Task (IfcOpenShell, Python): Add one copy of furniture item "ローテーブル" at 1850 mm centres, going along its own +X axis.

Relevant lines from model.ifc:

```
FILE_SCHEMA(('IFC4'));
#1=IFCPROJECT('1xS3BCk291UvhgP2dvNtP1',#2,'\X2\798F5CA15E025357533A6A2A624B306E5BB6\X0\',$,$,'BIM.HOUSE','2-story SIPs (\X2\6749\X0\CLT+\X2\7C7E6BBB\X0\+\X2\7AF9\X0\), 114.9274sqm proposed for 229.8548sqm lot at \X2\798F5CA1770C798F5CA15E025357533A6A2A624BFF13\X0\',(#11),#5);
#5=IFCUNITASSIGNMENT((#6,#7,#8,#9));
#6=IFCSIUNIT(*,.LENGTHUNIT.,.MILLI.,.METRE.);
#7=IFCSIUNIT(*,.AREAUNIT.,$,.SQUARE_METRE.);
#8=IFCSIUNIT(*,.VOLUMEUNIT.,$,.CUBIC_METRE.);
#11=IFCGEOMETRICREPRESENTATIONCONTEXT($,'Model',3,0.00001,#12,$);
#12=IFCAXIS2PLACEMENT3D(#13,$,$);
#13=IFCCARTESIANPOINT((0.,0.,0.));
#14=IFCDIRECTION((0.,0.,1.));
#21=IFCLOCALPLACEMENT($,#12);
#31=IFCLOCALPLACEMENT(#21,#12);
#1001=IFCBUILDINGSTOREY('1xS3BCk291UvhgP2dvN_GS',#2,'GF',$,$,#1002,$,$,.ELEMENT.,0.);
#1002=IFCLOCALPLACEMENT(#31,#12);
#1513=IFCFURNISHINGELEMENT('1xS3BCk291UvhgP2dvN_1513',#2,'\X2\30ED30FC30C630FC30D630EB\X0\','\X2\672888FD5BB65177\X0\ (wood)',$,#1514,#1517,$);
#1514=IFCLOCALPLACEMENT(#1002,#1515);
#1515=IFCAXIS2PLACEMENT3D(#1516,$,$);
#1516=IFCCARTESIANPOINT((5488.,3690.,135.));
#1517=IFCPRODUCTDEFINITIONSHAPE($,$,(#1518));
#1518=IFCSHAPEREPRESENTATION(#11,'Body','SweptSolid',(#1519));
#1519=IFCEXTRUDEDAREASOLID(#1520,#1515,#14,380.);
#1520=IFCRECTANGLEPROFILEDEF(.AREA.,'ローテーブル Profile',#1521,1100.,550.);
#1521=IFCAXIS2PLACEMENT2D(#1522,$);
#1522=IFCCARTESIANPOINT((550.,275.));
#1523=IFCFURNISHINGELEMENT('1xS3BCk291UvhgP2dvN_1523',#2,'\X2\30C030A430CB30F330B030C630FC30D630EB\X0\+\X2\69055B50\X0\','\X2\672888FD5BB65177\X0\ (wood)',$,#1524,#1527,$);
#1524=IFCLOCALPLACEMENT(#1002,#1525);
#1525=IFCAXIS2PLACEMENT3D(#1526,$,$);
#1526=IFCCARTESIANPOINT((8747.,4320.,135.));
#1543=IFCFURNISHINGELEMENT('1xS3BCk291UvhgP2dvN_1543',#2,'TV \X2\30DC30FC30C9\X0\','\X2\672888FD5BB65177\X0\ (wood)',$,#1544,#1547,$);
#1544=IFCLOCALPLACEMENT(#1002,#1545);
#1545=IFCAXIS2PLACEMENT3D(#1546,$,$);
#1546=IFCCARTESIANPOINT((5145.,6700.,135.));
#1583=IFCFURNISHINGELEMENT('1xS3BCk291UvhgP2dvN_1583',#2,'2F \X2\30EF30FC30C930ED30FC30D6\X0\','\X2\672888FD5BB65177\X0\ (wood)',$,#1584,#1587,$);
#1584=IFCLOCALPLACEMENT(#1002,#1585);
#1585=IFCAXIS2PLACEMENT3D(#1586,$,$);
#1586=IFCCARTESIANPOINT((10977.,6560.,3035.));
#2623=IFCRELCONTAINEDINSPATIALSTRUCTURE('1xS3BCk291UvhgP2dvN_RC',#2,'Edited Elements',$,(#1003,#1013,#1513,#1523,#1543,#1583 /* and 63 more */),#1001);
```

```python
import ifcopenshell
import ifcopenshell.api.geometry
import ifcopenshell.api.root
import ifcopenshell.util.element
import ifcopenshell.util.placement
import ifcopenshell.util.unit

model = ifcopenshell.open("model.ifc")
unit_scale = ifcopenshell.util.unit.calculate_unit_scale(model)


def reuse_history(source, copy):
    """copy_class also copies each property set's owner history, people and application; keep the originals."""
    for rel in copy.IsDefinedBy:
        if rel.is_a("IfcRelDefinesByProperties") and (history := rel.RelatingPropertyDefinition.OwnerHistory):
            rel.RelatingPropertyDefinition.OwnerHistory = source.OwnerHistory
            ifcopenshell.util.element.remove_deep2(model, history)


source = model.by_guid("1xS3BCk291UvhgP2dvN_1513")
base = ifcopenshell.util.placement.get_local_placement(source.ObjectPlacement)
step = base[:3, 0] * 1.85 / unit_scale

for i in range(1, 2):
    copy = ifcopenshell.api.root.copy_class(model, product=source)
    copy.Representation = ifcopenshell.util.element.copy_deep(
        model, source.Representation, exclude=["IfcGeometricRepresentationContext", "IfcRepresentationMap"]
    )
    reuse_history(source, copy)
    matrix = base.copy()
    matrix[:3, 3] += i * step
    print("added at", matrix[:3, 3].round(3) + 0.0)
    ifcopenshell.api.geometry.edit_object_placement(model, product=copy, matrix=matrix, is_si=False)

model.write("model_rev.ifc")
```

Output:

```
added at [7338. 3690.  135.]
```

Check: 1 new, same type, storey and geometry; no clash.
